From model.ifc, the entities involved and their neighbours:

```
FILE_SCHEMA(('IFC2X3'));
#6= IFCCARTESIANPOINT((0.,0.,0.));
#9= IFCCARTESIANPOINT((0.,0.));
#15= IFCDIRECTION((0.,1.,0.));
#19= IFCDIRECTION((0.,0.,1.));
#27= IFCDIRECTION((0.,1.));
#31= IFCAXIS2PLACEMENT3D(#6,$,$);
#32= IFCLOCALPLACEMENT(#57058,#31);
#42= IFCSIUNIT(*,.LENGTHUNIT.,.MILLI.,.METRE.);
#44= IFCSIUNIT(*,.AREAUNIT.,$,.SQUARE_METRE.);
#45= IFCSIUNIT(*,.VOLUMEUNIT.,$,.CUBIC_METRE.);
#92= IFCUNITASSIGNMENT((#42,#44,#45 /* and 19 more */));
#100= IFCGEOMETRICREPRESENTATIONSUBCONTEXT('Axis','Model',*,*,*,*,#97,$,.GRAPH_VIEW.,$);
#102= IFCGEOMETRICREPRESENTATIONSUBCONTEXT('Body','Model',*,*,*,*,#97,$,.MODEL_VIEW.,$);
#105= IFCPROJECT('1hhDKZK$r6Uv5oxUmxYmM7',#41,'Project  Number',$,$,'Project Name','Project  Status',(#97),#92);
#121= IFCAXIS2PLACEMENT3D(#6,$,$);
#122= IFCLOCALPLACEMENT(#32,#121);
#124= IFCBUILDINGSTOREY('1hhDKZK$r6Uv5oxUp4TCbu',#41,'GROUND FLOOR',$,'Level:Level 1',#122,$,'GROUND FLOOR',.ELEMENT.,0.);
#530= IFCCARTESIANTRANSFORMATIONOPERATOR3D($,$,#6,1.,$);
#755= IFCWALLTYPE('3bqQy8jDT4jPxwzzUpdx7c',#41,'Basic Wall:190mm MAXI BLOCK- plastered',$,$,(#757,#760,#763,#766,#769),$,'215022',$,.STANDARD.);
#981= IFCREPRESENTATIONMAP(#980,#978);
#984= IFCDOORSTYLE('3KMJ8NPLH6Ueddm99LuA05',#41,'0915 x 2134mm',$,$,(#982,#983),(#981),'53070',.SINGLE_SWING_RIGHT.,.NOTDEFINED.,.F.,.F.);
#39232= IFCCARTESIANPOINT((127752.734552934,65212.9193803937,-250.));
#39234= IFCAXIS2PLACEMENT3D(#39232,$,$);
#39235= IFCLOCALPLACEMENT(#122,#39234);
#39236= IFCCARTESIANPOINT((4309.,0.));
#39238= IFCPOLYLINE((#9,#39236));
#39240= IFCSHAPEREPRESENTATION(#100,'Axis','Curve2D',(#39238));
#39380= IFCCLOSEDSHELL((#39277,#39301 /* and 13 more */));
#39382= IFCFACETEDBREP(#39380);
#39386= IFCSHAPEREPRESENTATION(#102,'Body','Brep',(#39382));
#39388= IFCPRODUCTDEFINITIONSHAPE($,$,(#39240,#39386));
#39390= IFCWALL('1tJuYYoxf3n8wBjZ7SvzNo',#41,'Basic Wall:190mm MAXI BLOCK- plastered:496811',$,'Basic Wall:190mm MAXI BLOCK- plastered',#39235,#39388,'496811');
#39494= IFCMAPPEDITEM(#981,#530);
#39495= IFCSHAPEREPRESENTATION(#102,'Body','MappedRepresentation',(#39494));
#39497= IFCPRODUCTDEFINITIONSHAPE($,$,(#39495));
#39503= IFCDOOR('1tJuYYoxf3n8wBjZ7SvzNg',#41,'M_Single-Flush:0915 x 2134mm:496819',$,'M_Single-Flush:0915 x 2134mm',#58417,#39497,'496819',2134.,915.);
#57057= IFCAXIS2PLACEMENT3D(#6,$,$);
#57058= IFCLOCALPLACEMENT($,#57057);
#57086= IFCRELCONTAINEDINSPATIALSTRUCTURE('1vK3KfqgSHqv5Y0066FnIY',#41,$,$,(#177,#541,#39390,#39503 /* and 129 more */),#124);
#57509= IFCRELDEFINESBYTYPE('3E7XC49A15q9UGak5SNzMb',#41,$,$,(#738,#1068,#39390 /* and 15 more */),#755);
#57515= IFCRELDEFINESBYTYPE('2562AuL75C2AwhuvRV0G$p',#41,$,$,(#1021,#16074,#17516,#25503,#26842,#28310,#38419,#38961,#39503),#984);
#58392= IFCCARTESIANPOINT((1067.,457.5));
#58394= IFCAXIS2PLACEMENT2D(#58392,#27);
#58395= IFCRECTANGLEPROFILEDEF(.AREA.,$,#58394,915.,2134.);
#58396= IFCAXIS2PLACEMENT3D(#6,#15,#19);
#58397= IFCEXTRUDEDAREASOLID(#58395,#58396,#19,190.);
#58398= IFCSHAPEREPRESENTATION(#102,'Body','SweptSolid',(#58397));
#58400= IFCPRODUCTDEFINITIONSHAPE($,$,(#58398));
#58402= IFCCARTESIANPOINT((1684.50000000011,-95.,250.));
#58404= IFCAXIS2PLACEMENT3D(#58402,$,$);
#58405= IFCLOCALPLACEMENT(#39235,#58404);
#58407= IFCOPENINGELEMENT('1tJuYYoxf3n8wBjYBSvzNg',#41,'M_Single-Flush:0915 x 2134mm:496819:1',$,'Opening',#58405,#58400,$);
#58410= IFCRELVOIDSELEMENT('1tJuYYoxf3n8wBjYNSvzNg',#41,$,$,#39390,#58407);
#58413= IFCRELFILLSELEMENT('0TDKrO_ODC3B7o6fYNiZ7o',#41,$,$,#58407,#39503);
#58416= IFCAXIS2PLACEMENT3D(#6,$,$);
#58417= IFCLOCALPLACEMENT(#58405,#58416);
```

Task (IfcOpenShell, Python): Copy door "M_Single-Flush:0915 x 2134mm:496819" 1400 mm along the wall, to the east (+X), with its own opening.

```python
import ifcopenshell
import ifcopenshell.api.feature
import ifcopenshell.api.geometry
import ifcopenshell.api.root
import ifcopenshell.geom
import ifcopenshell.util.element
import ifcopenshell.util.placement
import ifcopenshell.util.shape
import ifcopenshell.util.unit

model = ifcopenshell.open("model.ifc")
unit_scale = ifcopenshell.util.unit.calculate_unit_scale(model)
settings = ifcopenshell.geom.settings()


def volume(element):
    """Net volume in cubic metres, openings subtracted."""
    shape = ifcopenshell.geom.create_shape(settings, element)
    return ifcopenshell.util.shape.get_volume(shape.geometry)


def reuse_history(source, copy):
    """copy_class also copies each property set's owner history, people and application; keep the originals."""
    for rel in copy.IsDefinedBy:
        if rel.is_a("IfcRelDefinesByProperties") and (history := rel.RelatingPropertyDefinition.OwnerHistory):
            rel.RelatingPropertyDefinition.OwnerHistory = source.OwnerHistory
            ifcopenshell.util.element.remove_deep2(model, history)


door = model.by_guid("1tJuYYoxf3n8wBjZ7SvzNg")
opening = door.FillsVoids[0].RelatingOpeningElement
wall = opening.VoidsElements[0].RelatingBuildingElement
before = volume(wall)
shift = ifcopenshell.util.placement.get_local_placement(wall.ObjectPlacement)[:3, 0] * 1.4 / unit_scale

# copy_class copies the void relationship, type, container and properties, but no geometry.
new_opening = ifcopenshell.api.root.copy_class(model, product=opening)
new_opening.Representation = ifcopenshell.util.element.copy_deep(
    model, opening.Representation, exclude=["IfcGeometricRepresentationContext", "IfcRepresentationMap"]
)
new_opening.Name = "M_Single-Flush:0915 x 2134mm"
new_door = ifcopenshell.api.root.copy_class(model, product=door)
new_door.Representation = ifcopenshell.util.element.copy_deep(
    model, door.Representation, exclude=["IfcGeometricRepresentationContext", "IfcRepresentationMap"]
)
new_door.Name = "M_Single-Flush:0915 x 2134mm"
new_door.Tag = None
reuse_history(door, new_door)
fills = ifcopenshell.api.feature.add_filling(model, opening=new_opening, element=new_door)
fills.OwnerHistory = new_door.OwnerHistory  # required in IFC2X3

for old, new in ((opening, new_opening), (door, new_door)):
    matrix = ifcopenshell.util.placement.get_local_placement(old.ObjectPlacement)
    matrix[:3, 3] += shift
    ifcopenshell.api.geometry.edit_object_placement(model, product=new, matrix=matrix, is_si=False)

after = volume(wall)

print(f"wall volume {before:.3f} -> {after:.3f} m3")

model.write("model_v2.ifc")
```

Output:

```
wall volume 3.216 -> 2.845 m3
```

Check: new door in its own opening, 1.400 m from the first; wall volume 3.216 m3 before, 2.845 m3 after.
